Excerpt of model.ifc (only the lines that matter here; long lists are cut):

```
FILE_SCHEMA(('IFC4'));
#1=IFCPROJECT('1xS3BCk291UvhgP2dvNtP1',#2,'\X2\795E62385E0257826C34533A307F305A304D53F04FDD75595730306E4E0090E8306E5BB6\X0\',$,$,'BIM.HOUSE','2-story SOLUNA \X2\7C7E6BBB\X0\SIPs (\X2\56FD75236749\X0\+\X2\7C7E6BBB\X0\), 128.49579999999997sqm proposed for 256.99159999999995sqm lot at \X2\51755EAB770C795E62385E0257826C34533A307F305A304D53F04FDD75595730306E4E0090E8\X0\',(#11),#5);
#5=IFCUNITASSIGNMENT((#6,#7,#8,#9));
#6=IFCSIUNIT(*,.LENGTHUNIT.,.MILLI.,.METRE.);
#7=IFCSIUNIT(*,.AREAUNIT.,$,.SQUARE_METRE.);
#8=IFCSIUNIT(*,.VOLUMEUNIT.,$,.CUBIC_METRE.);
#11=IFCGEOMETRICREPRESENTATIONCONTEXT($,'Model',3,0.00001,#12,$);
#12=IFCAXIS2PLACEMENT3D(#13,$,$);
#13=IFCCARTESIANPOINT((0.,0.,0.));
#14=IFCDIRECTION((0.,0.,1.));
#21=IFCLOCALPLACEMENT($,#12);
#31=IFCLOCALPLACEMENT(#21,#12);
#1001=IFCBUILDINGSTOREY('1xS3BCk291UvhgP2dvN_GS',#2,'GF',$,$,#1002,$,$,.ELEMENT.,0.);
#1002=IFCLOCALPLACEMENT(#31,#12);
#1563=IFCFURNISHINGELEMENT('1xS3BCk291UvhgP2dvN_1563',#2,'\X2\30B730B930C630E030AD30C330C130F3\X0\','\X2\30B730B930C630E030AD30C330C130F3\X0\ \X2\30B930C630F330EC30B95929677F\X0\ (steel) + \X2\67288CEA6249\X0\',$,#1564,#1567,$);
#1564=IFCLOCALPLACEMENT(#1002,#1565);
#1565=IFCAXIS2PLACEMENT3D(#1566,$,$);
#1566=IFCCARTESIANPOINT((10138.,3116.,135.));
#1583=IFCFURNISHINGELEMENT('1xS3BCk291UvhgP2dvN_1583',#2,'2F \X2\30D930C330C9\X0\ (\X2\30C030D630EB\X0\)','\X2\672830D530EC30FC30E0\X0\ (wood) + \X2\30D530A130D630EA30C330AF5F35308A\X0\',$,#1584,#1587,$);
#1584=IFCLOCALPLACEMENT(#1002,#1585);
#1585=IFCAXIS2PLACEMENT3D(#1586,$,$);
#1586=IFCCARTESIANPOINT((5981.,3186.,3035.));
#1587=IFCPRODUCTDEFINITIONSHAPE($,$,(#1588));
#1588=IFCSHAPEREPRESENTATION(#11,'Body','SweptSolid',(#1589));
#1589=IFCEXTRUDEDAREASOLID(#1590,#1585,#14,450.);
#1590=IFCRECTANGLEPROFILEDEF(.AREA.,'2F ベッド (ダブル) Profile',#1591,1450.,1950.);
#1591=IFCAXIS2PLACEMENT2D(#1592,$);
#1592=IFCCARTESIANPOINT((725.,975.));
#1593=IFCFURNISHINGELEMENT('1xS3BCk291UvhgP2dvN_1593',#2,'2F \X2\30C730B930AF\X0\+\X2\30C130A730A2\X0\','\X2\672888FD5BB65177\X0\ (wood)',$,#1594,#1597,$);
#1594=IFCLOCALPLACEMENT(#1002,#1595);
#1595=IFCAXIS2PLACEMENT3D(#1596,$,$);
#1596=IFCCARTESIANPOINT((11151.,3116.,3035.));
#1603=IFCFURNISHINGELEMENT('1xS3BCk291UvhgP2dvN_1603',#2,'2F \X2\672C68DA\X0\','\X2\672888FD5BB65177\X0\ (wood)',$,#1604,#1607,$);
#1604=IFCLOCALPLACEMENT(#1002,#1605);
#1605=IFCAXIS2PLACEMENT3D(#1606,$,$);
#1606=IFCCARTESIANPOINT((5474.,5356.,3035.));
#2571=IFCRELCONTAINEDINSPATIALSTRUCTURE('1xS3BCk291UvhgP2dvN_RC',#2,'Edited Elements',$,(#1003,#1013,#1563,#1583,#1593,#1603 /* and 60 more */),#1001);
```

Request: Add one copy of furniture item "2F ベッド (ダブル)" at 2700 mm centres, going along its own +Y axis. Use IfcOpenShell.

```python
import ifcopenshell
import ifcopenshell.api.geometry
import ifcopenshell.api.root
import ifcopenshell.util.element
import ifcopenshell.util.placement
import ifcopenshell.util.unit

model = ifcopenshell.open("model.ifc")
unit_scale = ifcopenshell.util.unit.calculate_unit_scale(model)


def reuse_history(source, copy):
    """copy_class also copies each property set's owner history, people and application; keep the originals."""
    for rel in copy.IsDefinedBy:
        if rel.is_a("IfcRelDefinesByProperties") and (history := rel.RelatingPropertyDefinition.OwnerHistory):
            rel.RelatingPropertyDefinition.OwnerHistory = source.OwnerHistory
            ifcopenshell.util.element.remove_deep2(model, history)


source = model.by_id(1583)
base = ifcopenshell.util.placement.get_local_placement(source.ObjectPlacement)
step = base[:3, 1] * 2.7 / unit_scale

for i in range(1, 2):
    copy = ifcopenshell.api.root.copy_class(model, product=source)
    copy.Representation = ifcopenshell.util.element.copy_deep(
        model, source.Representation, exclude=["IfcGeometricRepresentationContext", "IfcRepresentationMap"]
    )
    reuse_history(source, copy)
    matrix = base.copy()
    matrix[:3, 3] += i * step
    print("added at", matrix[:3, 3].round(3) + 0.0)
    ifcopenshell.api.geometry.edit_object_placement(model, product=copy, matrix=matrix, is_si=False)

model.write("model_updated.ifc")
```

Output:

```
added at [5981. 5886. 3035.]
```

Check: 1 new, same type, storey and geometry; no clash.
